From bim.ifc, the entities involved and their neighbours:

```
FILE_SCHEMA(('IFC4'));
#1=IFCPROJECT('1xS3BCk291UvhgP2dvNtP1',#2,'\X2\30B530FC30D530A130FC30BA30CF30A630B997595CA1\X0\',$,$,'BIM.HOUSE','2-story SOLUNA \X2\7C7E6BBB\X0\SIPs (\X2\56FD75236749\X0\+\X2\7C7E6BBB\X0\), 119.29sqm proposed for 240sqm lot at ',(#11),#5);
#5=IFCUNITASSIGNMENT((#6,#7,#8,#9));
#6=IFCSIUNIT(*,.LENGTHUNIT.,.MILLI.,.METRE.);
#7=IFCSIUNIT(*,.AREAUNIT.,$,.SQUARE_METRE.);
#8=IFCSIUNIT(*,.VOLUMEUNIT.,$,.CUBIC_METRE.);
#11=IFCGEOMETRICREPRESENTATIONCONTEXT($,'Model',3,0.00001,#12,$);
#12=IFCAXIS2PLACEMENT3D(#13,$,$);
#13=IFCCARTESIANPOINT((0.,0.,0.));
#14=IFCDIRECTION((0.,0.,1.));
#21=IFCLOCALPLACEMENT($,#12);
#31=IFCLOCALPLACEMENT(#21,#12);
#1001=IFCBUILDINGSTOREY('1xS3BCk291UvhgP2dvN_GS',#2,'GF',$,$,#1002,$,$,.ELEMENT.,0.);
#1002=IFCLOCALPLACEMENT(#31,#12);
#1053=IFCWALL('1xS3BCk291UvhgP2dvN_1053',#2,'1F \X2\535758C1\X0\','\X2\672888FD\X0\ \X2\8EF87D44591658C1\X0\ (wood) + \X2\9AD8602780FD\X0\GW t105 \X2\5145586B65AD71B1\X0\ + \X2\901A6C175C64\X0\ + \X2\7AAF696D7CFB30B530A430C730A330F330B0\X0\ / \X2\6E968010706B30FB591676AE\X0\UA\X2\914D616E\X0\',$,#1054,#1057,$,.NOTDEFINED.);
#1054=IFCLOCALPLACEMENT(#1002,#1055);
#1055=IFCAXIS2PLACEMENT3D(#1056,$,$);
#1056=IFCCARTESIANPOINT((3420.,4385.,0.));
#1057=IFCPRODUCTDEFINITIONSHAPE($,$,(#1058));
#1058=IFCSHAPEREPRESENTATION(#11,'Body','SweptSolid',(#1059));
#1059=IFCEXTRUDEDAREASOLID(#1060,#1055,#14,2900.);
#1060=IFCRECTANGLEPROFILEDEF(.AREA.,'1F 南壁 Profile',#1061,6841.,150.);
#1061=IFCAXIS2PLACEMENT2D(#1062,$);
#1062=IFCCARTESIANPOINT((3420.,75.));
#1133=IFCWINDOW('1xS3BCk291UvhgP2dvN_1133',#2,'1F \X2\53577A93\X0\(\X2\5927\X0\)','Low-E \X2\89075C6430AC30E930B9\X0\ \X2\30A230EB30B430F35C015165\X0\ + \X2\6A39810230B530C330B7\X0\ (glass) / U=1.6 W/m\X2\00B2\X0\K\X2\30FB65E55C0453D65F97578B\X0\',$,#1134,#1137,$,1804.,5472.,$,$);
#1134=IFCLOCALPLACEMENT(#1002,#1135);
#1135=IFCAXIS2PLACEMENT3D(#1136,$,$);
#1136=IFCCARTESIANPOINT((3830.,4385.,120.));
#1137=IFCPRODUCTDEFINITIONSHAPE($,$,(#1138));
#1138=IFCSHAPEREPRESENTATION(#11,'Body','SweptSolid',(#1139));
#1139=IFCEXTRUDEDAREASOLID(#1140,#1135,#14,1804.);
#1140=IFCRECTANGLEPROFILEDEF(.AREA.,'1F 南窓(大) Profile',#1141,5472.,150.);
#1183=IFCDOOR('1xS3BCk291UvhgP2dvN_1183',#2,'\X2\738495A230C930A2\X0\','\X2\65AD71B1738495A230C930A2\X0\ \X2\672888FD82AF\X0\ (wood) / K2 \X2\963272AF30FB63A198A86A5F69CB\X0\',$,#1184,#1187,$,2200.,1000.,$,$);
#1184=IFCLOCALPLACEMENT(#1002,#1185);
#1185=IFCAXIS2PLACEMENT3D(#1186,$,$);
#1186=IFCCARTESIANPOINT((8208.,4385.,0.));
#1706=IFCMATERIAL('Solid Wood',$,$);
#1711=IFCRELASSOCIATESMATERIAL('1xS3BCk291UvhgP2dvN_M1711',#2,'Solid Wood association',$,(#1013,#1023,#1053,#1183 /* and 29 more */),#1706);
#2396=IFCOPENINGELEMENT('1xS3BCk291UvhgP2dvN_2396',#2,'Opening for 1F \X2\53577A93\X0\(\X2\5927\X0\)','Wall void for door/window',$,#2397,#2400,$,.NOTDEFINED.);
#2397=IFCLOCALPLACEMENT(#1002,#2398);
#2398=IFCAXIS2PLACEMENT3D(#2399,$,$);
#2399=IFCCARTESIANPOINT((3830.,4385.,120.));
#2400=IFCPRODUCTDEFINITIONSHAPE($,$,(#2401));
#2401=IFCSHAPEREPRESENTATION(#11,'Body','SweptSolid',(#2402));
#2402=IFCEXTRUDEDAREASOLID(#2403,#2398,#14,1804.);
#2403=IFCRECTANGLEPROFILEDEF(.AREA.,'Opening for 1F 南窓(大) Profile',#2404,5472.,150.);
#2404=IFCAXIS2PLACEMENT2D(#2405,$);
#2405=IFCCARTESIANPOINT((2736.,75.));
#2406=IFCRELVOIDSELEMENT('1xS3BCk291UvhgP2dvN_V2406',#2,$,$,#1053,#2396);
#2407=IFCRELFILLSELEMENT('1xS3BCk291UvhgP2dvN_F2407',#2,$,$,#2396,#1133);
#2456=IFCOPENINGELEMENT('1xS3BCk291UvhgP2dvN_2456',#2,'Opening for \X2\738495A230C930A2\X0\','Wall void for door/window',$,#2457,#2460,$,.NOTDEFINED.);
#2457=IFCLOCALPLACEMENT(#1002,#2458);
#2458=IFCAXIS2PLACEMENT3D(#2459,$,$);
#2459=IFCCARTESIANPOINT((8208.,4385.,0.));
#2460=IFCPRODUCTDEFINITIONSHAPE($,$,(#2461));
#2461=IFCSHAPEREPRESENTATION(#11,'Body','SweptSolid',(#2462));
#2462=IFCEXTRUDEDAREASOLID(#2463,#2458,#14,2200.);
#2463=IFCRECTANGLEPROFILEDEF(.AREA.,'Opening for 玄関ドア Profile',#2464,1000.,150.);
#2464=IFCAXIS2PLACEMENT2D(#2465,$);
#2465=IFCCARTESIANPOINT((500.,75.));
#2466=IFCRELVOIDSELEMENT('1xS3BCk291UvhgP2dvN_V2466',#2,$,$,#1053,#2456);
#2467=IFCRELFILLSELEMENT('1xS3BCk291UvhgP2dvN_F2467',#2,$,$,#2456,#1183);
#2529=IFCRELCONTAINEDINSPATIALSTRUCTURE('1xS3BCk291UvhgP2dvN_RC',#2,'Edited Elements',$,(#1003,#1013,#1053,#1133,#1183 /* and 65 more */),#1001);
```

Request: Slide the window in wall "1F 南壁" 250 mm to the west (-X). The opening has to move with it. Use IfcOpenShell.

```python
import ifcopenshell
import ifcopenshell.api.geometry
import ifcopenshell.util.placement

model = ifcopenshell.open("bim.ifc")

window = model.by_guid("1xS3BCk291UvhgP2dvN_1133")
opening = window.FillsVoids[0].RelatingOpeningElement
wall = opening.VoidsElements[0].RelatingBuildingElement

wall_matrix = ifcopenshell.util.placement.get_local_placement(wall.ObjectPlacement)
shift = wall_matrix[:3, 0] * -250.0
before = ifcopenshell.util.placement.get_local_placement(window.ObjectPlacement)[:3, 3].copy()

# The window is not placed relative to its opening, so move both.
for product in (opening, window):
    matrix = ifcopenshell.util.placement.get_local_placement(product.ObjectPlacement)
    matrix[:3, 3] += shift
    ifcopenshell.api.geometry.edit_object_placement(model, product=product, matrix=matrix, is_si=False)

after = ifcopenshell.util.placement.get_local_placement(window.ObjectPlacement)[:3, 3]
print("window moved by", (after - before).round(3) + 0.0)

model.write("bim_edited.ifc")
```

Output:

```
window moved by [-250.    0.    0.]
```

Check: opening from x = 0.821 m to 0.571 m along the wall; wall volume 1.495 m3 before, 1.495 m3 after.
